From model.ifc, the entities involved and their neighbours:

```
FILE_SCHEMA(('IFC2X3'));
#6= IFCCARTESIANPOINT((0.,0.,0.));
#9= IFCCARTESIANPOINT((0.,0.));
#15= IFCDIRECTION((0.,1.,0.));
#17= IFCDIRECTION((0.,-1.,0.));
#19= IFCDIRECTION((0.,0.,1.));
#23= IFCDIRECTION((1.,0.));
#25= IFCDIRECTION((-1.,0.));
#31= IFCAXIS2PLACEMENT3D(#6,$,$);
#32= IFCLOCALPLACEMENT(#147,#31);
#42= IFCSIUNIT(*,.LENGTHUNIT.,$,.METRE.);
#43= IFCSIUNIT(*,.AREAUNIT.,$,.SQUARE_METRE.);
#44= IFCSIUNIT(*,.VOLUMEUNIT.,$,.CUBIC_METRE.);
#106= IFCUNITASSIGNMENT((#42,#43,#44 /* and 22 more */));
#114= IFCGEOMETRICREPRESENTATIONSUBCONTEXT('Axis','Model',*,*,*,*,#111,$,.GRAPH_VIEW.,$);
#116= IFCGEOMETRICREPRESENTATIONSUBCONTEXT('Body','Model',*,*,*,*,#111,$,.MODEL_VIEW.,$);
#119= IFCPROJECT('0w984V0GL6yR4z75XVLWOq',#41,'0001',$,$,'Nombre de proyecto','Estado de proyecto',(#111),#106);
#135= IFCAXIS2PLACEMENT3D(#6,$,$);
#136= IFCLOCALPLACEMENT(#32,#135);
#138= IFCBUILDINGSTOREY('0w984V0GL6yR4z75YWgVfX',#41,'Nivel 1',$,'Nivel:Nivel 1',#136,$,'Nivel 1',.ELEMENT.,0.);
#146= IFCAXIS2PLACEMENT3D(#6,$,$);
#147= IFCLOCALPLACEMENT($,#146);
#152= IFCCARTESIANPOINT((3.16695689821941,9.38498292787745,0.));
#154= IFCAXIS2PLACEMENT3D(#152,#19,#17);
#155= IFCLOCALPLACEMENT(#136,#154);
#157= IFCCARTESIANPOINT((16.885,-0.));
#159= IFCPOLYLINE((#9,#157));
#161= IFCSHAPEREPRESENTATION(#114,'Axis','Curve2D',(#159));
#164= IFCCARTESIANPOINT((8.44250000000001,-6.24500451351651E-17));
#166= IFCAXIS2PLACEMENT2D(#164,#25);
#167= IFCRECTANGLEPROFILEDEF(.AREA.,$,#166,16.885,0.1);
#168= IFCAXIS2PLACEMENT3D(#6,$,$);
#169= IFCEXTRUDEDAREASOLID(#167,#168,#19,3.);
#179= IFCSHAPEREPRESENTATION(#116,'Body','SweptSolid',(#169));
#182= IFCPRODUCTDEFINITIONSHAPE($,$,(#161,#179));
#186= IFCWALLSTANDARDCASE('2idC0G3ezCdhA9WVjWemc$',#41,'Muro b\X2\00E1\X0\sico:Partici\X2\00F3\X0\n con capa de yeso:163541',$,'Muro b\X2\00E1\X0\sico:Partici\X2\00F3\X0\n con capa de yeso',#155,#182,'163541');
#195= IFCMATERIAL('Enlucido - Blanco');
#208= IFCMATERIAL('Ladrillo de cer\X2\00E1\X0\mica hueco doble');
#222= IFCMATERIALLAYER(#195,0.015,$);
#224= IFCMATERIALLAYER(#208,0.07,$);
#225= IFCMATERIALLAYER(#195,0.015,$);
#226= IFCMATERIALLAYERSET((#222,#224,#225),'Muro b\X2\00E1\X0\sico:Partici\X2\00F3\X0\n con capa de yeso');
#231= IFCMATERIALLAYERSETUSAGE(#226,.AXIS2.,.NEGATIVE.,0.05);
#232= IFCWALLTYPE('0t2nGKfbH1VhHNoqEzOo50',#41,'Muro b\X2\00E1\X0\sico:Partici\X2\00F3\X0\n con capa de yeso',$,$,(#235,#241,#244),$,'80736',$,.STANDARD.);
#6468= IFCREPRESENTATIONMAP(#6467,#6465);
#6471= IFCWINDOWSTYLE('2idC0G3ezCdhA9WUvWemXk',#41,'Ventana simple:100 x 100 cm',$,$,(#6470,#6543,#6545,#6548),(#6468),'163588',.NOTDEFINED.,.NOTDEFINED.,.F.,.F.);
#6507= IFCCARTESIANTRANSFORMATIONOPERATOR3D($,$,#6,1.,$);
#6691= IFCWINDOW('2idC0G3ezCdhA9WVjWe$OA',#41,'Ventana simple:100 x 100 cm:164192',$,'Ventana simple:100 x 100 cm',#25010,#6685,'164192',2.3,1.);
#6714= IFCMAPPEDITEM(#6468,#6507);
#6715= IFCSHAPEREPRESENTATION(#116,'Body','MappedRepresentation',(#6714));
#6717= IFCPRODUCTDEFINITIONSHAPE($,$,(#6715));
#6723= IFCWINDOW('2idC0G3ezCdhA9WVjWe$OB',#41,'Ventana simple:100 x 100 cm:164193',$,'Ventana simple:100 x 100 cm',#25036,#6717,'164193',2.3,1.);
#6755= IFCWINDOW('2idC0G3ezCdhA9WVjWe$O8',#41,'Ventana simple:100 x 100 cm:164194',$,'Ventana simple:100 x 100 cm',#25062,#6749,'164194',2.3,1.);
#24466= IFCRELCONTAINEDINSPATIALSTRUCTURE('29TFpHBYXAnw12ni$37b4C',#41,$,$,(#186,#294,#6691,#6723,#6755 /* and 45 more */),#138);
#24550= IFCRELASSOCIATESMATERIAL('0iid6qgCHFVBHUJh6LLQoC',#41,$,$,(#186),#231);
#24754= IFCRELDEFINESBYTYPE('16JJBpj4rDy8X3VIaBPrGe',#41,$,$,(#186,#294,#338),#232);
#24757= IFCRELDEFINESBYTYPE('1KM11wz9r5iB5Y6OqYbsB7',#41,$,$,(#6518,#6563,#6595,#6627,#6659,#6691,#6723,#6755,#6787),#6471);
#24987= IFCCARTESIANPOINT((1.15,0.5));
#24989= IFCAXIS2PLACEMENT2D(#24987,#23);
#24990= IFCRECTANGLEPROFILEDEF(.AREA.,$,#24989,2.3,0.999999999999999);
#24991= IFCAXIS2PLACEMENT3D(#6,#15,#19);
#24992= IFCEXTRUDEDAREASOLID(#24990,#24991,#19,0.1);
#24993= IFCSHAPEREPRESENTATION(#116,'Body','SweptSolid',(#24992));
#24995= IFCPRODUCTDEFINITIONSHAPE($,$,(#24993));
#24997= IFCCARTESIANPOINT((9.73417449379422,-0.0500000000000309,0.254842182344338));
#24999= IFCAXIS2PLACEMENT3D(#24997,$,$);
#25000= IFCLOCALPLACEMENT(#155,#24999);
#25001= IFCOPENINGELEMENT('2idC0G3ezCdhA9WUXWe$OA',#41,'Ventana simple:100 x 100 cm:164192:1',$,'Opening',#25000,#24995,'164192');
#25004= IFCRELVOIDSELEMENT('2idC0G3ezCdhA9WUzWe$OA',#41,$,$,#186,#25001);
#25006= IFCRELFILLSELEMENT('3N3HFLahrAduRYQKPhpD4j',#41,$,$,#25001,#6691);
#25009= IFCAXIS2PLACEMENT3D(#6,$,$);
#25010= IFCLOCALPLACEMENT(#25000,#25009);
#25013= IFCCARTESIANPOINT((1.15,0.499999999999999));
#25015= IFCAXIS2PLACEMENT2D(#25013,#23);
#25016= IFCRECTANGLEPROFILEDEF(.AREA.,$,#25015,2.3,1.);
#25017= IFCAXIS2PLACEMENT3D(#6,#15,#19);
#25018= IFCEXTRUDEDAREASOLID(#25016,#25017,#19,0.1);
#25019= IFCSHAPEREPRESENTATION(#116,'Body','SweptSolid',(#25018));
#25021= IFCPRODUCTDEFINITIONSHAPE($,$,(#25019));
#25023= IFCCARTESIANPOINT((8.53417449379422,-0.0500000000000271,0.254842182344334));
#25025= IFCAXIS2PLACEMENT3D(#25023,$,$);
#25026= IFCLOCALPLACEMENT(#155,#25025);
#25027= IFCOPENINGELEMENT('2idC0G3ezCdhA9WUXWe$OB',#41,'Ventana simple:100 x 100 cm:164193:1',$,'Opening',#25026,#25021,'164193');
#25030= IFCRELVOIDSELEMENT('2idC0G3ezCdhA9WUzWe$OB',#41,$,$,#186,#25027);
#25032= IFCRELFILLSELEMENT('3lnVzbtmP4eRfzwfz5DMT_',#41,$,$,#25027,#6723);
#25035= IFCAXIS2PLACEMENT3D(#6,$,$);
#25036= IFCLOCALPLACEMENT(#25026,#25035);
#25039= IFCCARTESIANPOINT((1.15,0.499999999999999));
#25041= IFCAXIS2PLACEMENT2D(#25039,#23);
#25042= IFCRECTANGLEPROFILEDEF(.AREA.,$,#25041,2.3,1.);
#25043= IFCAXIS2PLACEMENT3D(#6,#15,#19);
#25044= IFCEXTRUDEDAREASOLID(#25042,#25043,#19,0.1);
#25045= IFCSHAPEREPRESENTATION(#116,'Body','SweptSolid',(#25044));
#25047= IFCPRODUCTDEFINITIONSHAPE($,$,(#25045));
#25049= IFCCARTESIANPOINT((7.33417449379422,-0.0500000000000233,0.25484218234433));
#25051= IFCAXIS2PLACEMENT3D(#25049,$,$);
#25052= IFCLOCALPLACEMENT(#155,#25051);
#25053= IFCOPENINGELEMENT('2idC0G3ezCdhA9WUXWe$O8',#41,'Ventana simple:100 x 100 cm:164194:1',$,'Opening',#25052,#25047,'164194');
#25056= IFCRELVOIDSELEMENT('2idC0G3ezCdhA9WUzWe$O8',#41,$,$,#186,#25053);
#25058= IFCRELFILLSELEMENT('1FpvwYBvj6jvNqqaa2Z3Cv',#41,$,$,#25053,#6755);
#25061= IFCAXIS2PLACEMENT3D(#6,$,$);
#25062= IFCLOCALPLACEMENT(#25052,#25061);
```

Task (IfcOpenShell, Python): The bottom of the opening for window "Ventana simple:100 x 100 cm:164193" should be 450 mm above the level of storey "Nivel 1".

```python
import numpy as np
import ifcopenshell
import ifcopenshell.api.geometry
import ifcopenshell.geom
import ifcopenshell.util.element
import ifcopenshell.util.placement
import ifcopenshell.util.shape
import ifcopenshell.util.unit

model = ifcopenshell.open("model.ifc")
unit_scale = ifcopenshell.util.unit.calculate_unit_scale(model)

window = model.by_id(6723)
opening = window.FillsVoids[0].RelatingOpeningElement
storey = ifcopenshell.util.element.get_container(window, ifc_class="IfcBuildingStorey")
level = ifcopenshell.util.placement.get_local_placement(storey.ObjectPlacement)[2, 3]

# The opening's origin need not be at the sill, so measure its lowest point.
shape = ifcopenshell.geom.create_shape(ifcopenshell.geom.settings(), opening)
bottom = ifcopenshell.util.shape.get_shape_bottom_elevation(shape, shape.geometry) / unit_scale
dz = level + 0.45 - bottom

shift = np.array([0.0, 0.0, dz])
# The window is placed relative to its opening, so it follows when the opening moves.
matrix = ifcopenshell.util.placement.get_local_placement(opening.ObjectPlacement)
matrix[:3, 3] += shift
ifcopenshell.api.geometry.edit_object_placement(
    model, product=opening, matrix=matrix, is_si=False, should_transform_children=True
)

print(f"moved by {dz * unit_scale:+.3f} m")

model.write("model_v2.ifc")
```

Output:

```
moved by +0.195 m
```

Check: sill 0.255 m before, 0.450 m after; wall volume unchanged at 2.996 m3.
